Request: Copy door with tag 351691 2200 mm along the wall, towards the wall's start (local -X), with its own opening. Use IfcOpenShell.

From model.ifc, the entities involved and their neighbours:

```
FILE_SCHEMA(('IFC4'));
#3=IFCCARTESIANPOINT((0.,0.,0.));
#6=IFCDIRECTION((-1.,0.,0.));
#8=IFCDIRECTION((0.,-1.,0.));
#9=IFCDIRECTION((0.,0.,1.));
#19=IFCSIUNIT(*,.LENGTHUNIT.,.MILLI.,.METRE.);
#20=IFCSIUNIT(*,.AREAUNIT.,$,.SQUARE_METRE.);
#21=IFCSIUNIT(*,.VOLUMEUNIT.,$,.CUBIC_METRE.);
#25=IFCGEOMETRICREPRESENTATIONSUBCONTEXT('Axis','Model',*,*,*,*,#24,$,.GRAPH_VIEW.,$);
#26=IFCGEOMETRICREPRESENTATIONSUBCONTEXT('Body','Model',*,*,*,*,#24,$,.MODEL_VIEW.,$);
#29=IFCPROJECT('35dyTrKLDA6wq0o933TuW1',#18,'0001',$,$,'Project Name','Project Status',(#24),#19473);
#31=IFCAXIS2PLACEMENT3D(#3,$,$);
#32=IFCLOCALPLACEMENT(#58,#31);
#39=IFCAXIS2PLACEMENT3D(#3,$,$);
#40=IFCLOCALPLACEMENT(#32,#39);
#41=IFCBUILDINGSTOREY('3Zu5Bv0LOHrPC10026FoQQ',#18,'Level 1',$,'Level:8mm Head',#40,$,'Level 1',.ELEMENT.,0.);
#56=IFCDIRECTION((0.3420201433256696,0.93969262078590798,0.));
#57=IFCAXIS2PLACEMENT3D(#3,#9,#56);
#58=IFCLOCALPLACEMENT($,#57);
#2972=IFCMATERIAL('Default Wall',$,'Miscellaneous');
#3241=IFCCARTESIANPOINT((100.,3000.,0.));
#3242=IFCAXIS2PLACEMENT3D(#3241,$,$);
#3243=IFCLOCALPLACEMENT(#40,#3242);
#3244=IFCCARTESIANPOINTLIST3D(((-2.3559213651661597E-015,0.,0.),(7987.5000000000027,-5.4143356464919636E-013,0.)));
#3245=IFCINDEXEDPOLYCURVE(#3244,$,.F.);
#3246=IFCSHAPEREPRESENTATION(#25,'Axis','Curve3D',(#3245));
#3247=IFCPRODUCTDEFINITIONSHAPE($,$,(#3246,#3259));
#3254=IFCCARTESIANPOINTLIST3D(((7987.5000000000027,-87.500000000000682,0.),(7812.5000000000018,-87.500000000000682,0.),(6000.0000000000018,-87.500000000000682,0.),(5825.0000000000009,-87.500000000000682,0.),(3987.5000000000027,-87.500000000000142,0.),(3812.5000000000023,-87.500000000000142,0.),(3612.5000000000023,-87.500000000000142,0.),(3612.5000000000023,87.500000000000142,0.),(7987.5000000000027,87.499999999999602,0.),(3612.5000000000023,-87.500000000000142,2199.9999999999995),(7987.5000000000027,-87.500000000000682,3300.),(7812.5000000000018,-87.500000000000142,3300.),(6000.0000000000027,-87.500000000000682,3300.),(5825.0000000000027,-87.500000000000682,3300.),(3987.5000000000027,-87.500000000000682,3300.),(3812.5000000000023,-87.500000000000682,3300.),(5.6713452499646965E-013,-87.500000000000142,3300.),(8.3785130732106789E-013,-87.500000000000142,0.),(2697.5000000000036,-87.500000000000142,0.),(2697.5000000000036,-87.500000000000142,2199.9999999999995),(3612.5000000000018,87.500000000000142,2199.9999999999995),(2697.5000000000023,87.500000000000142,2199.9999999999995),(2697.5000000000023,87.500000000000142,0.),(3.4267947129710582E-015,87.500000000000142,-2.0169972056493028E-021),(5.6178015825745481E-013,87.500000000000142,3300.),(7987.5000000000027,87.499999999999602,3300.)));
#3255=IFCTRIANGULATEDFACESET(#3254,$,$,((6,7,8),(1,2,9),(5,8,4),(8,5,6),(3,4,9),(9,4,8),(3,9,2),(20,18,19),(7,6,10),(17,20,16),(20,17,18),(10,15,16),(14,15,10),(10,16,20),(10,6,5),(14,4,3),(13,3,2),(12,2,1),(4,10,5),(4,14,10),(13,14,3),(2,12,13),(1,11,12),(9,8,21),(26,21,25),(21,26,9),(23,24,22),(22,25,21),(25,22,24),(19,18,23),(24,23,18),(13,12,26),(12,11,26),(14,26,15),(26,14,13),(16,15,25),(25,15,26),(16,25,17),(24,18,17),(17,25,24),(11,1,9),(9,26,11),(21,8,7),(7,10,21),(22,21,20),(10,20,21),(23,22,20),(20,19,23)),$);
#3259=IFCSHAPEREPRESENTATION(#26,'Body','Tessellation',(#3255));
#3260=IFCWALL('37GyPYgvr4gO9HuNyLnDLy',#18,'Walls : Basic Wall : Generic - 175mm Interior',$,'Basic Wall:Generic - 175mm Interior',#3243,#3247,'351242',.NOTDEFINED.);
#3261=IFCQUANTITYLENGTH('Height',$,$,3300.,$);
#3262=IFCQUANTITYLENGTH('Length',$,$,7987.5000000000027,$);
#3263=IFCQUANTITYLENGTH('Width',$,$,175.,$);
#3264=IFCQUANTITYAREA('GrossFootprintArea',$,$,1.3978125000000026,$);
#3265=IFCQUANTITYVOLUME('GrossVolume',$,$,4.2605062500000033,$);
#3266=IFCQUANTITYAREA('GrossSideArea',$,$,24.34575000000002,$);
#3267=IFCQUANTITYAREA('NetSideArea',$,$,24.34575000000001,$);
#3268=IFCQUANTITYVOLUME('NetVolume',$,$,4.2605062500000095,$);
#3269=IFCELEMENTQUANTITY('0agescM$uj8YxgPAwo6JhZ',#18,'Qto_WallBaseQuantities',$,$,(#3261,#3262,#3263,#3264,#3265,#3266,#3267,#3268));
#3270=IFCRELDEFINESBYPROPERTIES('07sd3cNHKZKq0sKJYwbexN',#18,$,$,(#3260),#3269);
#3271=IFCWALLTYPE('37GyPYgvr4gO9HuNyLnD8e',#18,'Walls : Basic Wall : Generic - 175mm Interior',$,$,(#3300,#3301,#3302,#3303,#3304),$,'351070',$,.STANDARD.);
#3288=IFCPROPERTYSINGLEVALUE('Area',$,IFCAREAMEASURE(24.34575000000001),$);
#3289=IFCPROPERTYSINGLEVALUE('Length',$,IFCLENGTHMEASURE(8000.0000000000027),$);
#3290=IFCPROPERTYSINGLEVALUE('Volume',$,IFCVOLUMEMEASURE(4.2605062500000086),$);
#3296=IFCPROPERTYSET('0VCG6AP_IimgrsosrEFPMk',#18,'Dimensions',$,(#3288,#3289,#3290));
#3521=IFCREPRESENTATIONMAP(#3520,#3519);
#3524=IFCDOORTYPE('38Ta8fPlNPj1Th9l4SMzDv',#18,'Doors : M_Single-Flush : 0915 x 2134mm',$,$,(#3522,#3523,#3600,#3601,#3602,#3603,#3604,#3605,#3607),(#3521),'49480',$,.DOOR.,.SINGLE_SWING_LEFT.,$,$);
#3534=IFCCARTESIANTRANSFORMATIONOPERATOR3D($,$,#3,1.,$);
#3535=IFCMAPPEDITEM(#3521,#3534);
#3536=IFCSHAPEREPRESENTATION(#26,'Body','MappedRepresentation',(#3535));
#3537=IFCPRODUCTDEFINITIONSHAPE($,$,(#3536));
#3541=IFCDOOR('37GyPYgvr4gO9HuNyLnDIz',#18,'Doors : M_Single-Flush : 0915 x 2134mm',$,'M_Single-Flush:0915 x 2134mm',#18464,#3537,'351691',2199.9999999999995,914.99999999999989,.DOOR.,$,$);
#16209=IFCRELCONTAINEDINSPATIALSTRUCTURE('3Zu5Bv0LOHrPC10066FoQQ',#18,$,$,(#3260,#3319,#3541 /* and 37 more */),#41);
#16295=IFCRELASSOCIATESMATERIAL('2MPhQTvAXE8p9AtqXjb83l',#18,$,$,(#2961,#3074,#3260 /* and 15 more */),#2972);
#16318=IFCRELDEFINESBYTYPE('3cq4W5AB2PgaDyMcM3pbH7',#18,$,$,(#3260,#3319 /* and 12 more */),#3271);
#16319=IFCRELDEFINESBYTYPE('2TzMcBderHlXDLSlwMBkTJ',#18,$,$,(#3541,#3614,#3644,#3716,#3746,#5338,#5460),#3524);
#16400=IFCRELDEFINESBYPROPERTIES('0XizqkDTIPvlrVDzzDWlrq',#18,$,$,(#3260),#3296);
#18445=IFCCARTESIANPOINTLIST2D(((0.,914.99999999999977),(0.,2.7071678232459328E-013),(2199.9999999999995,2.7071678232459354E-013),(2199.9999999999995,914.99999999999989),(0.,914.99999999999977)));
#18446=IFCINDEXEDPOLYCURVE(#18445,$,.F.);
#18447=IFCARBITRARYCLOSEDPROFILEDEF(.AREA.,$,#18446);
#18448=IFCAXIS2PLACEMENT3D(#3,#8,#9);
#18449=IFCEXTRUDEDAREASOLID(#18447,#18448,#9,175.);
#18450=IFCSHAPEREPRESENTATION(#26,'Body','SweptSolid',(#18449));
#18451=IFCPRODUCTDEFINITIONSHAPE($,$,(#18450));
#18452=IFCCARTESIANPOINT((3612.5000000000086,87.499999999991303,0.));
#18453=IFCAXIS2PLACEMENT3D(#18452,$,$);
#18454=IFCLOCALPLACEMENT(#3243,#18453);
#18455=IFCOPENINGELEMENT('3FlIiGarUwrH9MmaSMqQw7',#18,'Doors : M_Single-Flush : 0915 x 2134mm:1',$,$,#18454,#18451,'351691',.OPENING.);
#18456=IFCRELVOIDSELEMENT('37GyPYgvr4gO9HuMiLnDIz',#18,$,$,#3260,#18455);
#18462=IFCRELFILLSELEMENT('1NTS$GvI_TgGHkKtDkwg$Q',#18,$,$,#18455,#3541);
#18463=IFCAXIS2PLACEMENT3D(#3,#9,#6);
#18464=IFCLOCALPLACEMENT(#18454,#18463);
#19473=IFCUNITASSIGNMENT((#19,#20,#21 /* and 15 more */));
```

```python
import ifcopenshell
import ifcopenshell.api.feature
import ifcopenshell.api.geometry
import ifcopenshell.api.pset
import ifcopenshell.api.root
import ifcopenshell.geom
import ifcopenshell.util.element
import ifcopenshell.util.placement
import ifcopenshell.util.shape
import ifcopenshell.util.unit

model = ifcopenshell.open("model.ifc")
unit_scale = ifcopenshell.util.unit.calculate_unit_scale(model)
area_scale = ifcopenshell.util.unit.calculate_unit_scale(model, "AREAUNIT")
volume_scale = ifcopenshell.util.unit.calculate_unit_scale(model, "VOLUMEUNIT")
settings = ifcopenshell.geom.settings()


def volume(element):
    """Net volume in cubic metres, openings subtracted."""
    shape = ifcopenshell.geom.create_shape(settings, element)
    return ifcopenshell.util.shape.get_volume(shape.geometry)


def reuse_history(source, copy):
    """copy_class also copies each property set's owner history, people and application; keep the originals."""
    for rel in copy.IsDefinedBy:
        if rel.is_a("IfcRelDefinesByProperties") and (history := rel.RelatingPropertyDefinition.OwnerHistory):
            rel.RelatingPropertyDefinition.OwnerHistory = source.OwnerHistory
            ifcopenshell.util.element.remove_deep2(model, history)


door = model.by_guid("37GyPYgvr4gO9HuNyLnDIz")
opening = door.FillsVoids[0].RelatingOpeningElement
wall = opening.VoidsElements[0].RelatingBuildingElement
before = volume(wall)
shift = ifcopenshell.util.placement.get_local_placement(wall.ObjectPlacement)[:3, 0] * -2.2 / unit_scale

# copy_class copies the void relationship, type, container and properties, but no geometry.
new_opening = ifcopenshell.api.root.copy_class(model, product=opening)
new_opening.Representation = ifcopenshell.util.element.copy_deep(
    model, opening.Representation, exclude=["IfcGeometricRepresentationContext", "IfcRepresentationMap"]
)
new_opening.Tag = None
reuse_history(opening, new_opening)
new_door = ifcopenshell.api.root.copy_class(model, product=door)
new_door.Representation = ifcopenshell.util.element.copy_deep(
    model, door.Representation, exclude=["IfcGeometricRepresentationContext", "IfcRepresentationMap"]
)
new_door.Tag = None
reuse_history(door, new_door)
ifcopenshell.api.feature.add_filling(model, opening=new_opening, element=new_door)

for old, new in ((opening, new_opening), (door, new_door)):
    matrix = ifcopenshell.util.placement.get_local_placement(old.ObjectPlacement)
    matrix[:3, 3] += shift
    ifcopenshell.api.geometry.edit_object_placement(model, product=new, matrix=matrix, is_si=False)

after = volume(wall)
thickness = 0.175  # wall thickness in metres

# Update the wall's stored quantities.
qto = model.by_id(ifcopenshell.util.element.get_pset(wall, "Qto_WallBaseQuantities", should_inherit=False)["id"])
ifcopenshell.api.pset.edit_qto(model, qto=qto, properties={
    "NetSideArea": after / thickness / area_scale,
    "NetVolume": after / volume_scale,
})
pset = model.by_id(ifcopenshell.util.element.get_pset(wall, "Dimensions", should_inherit=False)["id"])
ifcopenshell.api.pset.edit_pset(model, pset=pset, properties={
    "Area": model.create_entity("IfcAreaMeasure", after / thickness / area_scale),
    "Volume": model.create_entity("IfcVolumeMeasure", after / volume_scale),
})

print(f"wall volume {before:.3f} -> {after:.3f} m3")

model.write("model_updated.ifc")
```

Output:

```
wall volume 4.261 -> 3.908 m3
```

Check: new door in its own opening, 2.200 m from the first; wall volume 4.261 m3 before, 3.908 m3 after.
